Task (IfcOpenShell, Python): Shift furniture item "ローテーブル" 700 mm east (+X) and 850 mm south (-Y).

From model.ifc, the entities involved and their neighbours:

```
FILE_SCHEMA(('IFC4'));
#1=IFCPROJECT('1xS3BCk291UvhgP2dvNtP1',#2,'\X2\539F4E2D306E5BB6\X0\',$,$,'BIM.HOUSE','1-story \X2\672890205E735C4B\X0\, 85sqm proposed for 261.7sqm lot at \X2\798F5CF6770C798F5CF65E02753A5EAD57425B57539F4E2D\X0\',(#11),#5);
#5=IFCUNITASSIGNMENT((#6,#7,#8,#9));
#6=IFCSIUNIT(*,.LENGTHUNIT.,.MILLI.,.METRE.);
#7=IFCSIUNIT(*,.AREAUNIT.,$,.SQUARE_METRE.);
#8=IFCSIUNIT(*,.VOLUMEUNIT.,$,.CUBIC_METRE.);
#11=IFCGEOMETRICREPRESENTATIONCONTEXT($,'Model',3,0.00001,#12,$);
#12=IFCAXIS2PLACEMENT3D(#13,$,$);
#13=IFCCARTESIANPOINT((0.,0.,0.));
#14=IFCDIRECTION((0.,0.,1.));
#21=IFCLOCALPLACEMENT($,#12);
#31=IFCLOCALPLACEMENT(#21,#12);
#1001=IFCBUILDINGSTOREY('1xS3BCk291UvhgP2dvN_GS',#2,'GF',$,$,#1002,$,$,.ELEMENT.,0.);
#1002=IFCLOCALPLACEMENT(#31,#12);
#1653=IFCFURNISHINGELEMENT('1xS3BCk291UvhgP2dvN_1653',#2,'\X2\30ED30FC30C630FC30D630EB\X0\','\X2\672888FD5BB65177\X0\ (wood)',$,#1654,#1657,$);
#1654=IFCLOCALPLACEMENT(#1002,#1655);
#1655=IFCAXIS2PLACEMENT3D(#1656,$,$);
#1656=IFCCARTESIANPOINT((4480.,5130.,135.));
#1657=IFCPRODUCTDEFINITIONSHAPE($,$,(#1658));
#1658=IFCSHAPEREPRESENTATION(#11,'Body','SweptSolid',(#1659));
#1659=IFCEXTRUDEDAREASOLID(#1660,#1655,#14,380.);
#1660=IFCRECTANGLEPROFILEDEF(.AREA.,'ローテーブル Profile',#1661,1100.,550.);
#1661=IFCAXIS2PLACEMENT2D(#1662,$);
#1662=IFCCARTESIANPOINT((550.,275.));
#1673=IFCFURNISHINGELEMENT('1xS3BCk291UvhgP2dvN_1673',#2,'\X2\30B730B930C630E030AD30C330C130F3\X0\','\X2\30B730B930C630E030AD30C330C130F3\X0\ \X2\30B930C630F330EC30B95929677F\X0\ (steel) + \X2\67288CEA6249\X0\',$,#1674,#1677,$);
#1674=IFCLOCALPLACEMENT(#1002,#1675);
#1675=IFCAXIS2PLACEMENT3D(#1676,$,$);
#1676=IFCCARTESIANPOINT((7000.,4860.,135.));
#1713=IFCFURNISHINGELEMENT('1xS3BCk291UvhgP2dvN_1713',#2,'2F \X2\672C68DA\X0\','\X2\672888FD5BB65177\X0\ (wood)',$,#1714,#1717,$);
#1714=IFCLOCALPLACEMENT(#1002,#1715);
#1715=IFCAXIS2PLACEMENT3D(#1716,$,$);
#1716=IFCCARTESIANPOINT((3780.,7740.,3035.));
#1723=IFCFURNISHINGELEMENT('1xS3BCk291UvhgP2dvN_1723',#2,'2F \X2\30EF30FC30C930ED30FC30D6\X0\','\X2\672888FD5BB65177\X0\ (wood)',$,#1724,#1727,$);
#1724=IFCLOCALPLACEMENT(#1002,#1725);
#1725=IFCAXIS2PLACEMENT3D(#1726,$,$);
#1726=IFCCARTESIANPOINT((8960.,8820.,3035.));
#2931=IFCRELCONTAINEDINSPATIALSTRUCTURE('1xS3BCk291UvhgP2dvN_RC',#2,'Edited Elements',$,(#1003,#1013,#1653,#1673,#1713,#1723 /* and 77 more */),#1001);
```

```python
import ifcopenshell
import ifcopenshell.api.geometry
import ifcopenshell.util.placement
import ifcopenshell.util.unit

model = ifcopenshell.open("model.ifc")
unit_scale = ifcopenshell.util.unit.calculate_unit_scale(model)

item = model.by_id(1653)
matrix = ifcopenshell.util.placement.get_local_placement(item.ObjectPlacement)
matrix[0, 3] += 0.7 / unit_scale
matrix[1, 3] -= 0.85 / unit_scale
ifcopenshell.api.geometry.edit_object_placement(model, product=item, matrix=matrix, is_si=False)

print(ifcopenshell.util.placement.get_local_placement(item.ObjectPlacement).round(3) + 0.0)

model.write("model-out.ifc")
```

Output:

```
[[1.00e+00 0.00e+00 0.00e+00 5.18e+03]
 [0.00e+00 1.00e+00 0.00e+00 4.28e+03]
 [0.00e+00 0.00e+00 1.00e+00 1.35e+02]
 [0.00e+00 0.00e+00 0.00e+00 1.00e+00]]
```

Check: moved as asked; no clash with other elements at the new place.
